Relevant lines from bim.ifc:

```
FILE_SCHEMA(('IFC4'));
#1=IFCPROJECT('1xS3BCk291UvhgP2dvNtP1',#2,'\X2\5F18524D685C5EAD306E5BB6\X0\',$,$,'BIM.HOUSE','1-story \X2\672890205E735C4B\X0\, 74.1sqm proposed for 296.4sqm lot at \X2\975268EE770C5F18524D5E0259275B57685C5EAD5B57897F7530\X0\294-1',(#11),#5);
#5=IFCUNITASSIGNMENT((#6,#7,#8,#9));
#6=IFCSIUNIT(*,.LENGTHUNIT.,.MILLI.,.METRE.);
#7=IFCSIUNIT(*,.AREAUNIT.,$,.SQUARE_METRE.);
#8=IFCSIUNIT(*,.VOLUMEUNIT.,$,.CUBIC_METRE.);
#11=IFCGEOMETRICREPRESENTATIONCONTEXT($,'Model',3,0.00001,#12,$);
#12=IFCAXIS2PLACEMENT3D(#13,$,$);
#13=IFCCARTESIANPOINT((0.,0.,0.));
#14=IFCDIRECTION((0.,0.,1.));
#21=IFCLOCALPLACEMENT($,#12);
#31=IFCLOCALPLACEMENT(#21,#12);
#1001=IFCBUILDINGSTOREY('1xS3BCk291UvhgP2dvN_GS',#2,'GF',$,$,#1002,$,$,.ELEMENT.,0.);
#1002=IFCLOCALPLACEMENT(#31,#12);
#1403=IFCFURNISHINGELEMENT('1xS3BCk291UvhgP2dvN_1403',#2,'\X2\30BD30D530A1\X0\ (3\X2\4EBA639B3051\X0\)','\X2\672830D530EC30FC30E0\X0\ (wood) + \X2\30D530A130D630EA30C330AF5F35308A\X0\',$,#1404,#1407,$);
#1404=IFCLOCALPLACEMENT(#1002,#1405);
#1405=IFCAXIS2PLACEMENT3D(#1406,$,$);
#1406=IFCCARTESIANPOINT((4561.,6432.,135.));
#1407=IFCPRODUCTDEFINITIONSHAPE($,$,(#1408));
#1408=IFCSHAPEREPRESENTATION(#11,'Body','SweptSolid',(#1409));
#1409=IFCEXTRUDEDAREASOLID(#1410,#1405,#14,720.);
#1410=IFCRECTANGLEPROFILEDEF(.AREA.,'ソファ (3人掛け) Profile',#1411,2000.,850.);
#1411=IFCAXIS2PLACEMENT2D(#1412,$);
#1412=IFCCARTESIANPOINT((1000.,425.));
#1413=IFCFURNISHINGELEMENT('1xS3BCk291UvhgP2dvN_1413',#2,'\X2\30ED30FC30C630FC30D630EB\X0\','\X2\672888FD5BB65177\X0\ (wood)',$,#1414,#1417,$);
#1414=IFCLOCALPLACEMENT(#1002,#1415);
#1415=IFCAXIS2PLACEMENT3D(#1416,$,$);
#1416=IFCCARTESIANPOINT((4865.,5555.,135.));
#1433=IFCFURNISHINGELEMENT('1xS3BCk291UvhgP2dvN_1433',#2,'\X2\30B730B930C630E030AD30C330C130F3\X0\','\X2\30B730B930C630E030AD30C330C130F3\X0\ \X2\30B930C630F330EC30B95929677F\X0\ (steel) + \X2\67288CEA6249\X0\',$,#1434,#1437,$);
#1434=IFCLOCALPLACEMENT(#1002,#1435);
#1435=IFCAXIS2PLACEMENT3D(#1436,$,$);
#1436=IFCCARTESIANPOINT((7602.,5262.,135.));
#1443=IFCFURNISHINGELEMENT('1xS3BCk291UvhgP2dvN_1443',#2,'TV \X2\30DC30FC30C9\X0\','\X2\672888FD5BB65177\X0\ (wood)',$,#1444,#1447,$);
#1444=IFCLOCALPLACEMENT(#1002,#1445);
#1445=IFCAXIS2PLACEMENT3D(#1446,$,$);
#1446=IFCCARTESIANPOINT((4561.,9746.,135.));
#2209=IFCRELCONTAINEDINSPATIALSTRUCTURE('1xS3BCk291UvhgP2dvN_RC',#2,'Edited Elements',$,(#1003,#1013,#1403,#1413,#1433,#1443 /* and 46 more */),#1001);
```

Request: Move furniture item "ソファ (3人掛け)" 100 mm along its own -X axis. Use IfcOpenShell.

```python
import ifcopenshell
import ifcopenshell.api.geometry
import ifcopenshell.util.placement

model = ifcopenshell.open("bim.ifc")

item = model.by_id(1403)
matrix = ifcopenshell.util.placement.get_local_placement(item.ObjectPlacement)
matrix[:3, 3] -= matrix[:3, 0] * 100.0
ifcopenshell.api.geometry.edit_object_placement(model, product=item, matrix=matrix, is_si=False)

print(ifcopenshell.util.placement.get_local_placement(item.ObjectPlacement).round(3) + 0.0)

model.write("bim_updated.ifc")
```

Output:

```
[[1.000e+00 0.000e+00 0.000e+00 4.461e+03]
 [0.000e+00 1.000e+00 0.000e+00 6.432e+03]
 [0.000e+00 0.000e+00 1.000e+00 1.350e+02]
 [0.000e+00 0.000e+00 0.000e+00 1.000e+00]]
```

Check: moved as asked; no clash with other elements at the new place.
